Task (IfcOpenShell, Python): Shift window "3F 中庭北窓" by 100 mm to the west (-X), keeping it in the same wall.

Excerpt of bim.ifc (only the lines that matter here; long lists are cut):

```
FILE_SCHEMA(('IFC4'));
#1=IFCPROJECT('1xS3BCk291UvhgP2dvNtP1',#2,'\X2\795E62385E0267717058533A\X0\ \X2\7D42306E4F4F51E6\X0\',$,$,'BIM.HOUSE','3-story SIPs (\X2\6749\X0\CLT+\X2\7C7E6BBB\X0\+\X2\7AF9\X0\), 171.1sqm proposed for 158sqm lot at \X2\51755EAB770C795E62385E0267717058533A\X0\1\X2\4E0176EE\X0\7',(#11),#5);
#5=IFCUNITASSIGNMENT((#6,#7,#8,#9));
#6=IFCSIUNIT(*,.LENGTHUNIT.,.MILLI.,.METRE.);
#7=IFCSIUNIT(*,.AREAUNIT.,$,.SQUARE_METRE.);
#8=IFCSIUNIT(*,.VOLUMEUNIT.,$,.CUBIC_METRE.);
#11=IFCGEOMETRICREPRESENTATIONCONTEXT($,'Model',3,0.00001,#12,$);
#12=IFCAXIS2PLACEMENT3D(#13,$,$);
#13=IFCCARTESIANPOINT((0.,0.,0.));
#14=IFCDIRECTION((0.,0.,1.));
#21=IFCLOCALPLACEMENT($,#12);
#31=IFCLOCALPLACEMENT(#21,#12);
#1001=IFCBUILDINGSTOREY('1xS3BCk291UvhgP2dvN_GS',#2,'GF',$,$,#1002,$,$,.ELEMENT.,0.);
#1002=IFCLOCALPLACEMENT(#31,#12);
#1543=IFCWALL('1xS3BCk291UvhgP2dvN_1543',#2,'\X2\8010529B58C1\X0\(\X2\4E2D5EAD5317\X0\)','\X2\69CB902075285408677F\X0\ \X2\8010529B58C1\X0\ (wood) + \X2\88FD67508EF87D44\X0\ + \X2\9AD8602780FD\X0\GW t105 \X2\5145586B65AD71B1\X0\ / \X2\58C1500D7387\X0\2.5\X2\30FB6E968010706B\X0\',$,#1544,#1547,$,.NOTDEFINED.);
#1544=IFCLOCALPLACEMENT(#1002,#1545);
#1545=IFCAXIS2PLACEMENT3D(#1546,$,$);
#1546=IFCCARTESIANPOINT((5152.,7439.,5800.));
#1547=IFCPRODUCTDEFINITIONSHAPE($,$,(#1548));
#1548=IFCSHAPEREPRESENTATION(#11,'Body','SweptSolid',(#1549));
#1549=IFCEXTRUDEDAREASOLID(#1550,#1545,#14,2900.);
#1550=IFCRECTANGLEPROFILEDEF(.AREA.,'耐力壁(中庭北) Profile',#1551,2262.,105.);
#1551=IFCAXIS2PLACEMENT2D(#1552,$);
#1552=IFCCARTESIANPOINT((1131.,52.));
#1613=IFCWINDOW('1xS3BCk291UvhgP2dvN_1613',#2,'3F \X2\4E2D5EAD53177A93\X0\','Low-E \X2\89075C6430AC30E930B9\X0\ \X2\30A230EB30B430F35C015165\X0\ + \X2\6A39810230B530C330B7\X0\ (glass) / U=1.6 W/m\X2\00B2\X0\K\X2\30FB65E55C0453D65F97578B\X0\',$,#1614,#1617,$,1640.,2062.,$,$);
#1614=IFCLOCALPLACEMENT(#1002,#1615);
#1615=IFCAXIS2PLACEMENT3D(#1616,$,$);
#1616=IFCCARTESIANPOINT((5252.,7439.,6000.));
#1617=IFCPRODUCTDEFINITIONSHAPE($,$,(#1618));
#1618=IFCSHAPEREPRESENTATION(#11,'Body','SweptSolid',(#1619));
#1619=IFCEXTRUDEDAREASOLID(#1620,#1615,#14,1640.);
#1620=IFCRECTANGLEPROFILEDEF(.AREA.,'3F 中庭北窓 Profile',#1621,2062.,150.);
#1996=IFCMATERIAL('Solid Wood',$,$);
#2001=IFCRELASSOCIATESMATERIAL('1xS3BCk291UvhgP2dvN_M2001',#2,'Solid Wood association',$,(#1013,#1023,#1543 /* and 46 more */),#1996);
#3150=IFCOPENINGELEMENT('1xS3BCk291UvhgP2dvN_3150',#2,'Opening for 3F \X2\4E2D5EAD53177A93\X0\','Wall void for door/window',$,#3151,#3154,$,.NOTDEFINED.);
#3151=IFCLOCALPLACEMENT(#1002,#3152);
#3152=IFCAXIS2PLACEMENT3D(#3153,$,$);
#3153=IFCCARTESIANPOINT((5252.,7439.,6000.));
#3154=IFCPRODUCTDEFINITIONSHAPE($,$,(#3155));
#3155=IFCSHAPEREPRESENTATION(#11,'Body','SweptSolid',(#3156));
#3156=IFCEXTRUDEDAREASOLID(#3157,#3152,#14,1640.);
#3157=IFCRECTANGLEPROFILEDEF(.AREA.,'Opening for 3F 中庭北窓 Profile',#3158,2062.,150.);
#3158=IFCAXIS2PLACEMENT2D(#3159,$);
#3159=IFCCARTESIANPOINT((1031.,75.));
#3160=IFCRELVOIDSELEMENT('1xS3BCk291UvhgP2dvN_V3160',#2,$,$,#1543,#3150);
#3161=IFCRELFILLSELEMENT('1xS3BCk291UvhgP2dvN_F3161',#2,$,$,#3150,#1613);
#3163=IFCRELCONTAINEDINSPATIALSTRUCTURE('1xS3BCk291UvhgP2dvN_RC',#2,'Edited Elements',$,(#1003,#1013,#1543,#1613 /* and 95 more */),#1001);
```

```python
import ifcopenshell
import ifcopenshell.api.geometry
import ifcopenshell.util.placement
import ifcopenshell.util.unit

model = ifcopenshell.open("bim.ifc")
unit_scale = ifcopenshell.util.unit.calculate_unit_scale(model)

window = model.by_guid("1xS3BCk291UvhgP2dvN_1613")
opening = window.FillsVoids[0].RelatingOpeningElement
wall = opening.VoidsElements[0].RelatingBuildingElement

wall_matrix = ifcopenshell.util.placement.get_local_placement(wall.ObjectPlacement)
shift = wall_matrix[:3, 0] * -0.1 / unit_scale
before = ifcopenshell.util.placement.get_local_placement(window.ObjectPlacement)[:3, 3].copy()

# The window is not placed relative to its opening, so move both.
for product in (opening, window):
    matrix = ifcopenshell.util.placement.get_local_placement(product.ObjectPlacement)
    matrix[:3, 3] += shift
    ifcopenshell.api.geometry.edit_object_placement(model, product=product, matrix=matrix, is_si=False)

after = ifcopenshell.util.placement.get_local_placement(window.ObjectPlacement)[:3, 3]
print("window moved by", (after - before).round(3) + 0.0)

model.write("bim-out.ifc")
```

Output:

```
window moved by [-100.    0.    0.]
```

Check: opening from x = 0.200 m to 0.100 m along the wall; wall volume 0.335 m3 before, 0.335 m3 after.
